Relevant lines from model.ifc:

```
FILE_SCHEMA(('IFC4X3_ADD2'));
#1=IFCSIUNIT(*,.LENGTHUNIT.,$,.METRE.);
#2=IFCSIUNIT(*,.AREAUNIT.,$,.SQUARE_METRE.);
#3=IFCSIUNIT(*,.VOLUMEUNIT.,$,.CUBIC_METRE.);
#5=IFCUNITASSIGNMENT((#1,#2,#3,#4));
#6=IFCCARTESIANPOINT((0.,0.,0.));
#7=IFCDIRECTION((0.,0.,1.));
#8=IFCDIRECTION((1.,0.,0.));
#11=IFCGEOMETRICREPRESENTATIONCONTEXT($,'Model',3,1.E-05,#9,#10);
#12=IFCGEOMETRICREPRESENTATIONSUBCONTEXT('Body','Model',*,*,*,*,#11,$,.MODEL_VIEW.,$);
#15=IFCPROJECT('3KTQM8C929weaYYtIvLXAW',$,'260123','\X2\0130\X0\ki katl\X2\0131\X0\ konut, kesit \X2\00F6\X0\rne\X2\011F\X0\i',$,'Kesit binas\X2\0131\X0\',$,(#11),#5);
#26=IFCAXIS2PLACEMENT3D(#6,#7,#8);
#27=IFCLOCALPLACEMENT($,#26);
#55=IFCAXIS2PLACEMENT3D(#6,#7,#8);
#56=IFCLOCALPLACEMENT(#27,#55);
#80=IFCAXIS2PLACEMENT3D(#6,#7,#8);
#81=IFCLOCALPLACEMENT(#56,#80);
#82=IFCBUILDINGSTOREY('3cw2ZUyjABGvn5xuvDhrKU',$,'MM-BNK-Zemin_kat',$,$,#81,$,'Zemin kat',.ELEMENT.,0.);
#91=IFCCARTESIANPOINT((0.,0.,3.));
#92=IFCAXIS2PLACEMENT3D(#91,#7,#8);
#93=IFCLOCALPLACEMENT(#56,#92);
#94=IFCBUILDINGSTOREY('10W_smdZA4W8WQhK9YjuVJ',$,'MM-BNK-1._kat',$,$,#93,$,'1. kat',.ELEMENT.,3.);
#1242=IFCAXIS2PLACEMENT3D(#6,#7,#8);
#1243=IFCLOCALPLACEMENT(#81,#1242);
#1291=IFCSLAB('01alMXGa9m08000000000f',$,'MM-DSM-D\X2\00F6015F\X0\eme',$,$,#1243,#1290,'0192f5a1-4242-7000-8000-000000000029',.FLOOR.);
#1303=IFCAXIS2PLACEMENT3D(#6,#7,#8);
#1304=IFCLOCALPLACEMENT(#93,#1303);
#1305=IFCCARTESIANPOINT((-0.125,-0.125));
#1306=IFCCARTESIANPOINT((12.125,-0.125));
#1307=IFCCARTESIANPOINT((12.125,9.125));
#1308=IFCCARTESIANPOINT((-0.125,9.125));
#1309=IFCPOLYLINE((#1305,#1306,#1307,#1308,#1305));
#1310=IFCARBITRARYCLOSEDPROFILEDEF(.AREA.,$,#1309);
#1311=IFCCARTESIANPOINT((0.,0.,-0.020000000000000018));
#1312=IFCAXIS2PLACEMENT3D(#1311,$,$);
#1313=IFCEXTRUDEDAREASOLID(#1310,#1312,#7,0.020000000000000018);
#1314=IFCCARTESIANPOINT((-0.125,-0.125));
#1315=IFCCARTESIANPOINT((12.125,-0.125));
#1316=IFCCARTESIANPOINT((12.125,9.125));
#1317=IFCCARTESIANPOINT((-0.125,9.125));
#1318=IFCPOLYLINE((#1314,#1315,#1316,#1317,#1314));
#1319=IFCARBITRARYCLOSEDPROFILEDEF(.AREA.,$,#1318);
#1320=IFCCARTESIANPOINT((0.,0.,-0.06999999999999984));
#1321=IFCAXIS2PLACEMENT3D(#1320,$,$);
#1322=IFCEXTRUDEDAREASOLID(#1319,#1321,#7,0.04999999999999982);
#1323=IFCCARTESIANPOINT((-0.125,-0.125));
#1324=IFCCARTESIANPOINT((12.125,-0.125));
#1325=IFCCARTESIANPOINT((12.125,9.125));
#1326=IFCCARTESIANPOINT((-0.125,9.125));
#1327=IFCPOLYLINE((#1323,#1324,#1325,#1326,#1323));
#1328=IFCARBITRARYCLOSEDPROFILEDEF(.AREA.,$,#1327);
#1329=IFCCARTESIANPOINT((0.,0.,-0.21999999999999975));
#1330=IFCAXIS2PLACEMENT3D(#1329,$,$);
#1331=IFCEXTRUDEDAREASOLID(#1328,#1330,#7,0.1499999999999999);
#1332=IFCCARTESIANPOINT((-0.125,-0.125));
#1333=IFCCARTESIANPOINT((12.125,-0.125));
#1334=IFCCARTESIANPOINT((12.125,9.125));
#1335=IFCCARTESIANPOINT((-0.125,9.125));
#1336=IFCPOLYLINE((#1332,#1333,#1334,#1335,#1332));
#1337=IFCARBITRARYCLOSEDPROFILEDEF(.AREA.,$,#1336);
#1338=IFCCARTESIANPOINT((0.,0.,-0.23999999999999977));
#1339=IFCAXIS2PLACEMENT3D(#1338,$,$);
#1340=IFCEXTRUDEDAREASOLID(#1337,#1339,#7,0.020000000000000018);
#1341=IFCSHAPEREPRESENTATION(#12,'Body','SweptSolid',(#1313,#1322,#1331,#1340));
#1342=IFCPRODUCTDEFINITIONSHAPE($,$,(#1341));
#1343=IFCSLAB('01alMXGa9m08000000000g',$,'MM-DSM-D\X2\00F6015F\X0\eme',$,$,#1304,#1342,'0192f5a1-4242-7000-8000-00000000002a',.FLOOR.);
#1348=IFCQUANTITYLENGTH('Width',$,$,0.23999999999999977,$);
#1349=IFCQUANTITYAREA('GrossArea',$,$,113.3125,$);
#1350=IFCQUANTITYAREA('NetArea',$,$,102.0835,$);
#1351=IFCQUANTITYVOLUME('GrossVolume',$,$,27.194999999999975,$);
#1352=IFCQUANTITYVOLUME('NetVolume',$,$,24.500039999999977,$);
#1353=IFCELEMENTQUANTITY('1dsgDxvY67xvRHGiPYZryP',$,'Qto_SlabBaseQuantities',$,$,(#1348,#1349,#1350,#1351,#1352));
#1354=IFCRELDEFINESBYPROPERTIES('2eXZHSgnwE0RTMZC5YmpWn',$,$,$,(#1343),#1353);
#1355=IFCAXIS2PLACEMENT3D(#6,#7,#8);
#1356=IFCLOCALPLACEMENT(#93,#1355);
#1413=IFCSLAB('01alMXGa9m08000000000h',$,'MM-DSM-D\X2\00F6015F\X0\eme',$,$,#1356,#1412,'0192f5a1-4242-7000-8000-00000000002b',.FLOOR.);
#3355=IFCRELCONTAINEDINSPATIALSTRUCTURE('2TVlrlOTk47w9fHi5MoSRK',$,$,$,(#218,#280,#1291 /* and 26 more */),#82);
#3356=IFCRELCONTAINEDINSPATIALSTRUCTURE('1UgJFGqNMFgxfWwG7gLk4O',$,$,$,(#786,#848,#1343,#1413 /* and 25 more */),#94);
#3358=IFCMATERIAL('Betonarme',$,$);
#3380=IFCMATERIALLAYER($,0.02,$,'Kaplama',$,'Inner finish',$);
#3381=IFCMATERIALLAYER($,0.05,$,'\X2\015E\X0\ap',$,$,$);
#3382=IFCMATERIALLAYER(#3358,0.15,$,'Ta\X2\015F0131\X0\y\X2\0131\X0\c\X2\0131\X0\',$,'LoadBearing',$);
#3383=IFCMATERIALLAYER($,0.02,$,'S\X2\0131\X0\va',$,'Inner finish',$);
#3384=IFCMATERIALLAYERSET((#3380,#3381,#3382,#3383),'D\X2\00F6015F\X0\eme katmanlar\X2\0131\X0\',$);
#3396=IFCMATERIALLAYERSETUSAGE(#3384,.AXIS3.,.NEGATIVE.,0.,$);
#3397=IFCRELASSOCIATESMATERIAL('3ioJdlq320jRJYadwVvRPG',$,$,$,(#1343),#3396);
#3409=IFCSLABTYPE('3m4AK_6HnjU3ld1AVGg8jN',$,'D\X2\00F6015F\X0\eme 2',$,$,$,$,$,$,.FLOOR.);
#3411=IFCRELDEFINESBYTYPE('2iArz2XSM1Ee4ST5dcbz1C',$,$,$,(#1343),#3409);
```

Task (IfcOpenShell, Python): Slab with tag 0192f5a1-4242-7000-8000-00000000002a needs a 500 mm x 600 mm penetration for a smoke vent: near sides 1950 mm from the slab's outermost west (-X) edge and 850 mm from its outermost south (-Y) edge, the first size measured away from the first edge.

```python
import numpy as np
import ifcopenshell
import ifcopenshell.api.feature
import ifcopenshell.api.geometry
import ifcopenshell.api.pset
import ifcopenshell.api.root
import ifcopenshell.geom
import ifcopenshell.util.element
import ifcopenshell.util.placement
import ifcopenshell.util.representation
import ifcopenshell.util.shape
import ifcopenshell.util.unit

model = ifcopenshell.open("model.ifc")
unit_scale = ifcopenshell.util.unit.calculate_unit_scale(model)
area_scale = ifcopenshell.util.unit.calculate_unit_scale(model, "AREAUNIT")
volume_scale = ifcopenshell.util.unit.calculate_unit_scale(model, "VOLUMEUNIT")
settings = ifcopenshell.geom.settings()


def volume(element):
    """Net volume in cubic metres, openings subtracted."""
    shape = ifcopenshell.geom.create_shape(settings, element)
    return ifcopenshell.util.shape.get_volume(shape.geometry)


slab = model.by_guid("01alMXGa9m08000000000g")
before = volume(slab)

# Extent in the slab's own axes, in metres. The edges named are its -X and -Y sides.
slab_shape = ifcopenshell.geom.create_shape(settings, slab)
vertices = ifcopenshell.util.shape.get_vertices(slab_shape.geometry)
x_min, y_min, bottom = vertices.min(axis=0)
top = vertices[:, 2].max()

opening = ifcopenshell.api.root.create_entity(model, ifc_class="IfcOpeningElement", name="Smoke vent opening", predefined_type="OPENING")
context = ifcopenshell.util.representation.get_context(model, "Model", "Body", "MODEL_VIEW")
width, depth = 0.5, 0.6
outline = [(0.0, 0.0), (width, 0.0), (width, depth), (0.0, depth), (0.0, 0.0)]
# Overshoot both faces by 50 mm so the cut is clean.
shape = ifcopenshell.api.geometry.add_slab_representation(
    model, context=context, depth=top - bottom + 0.1, polyline=outline
)
ifcopenshell.api.geometry.assign_representation(model, product=opening, representation=shape)

matrix = ifcopenshell.util.placement.get_local_placement(slab.ObjectPlacement)
matrix[:, 3] = matrix @ np.append(np.array([x_min + 1.95, y_min + 0.85, bottom - 0.05]) / unit_scale, 1.0)
ifcopenshell.api.geometry.edit_object_placement(model, product=opening, matrix=matrix, is_si=False)
ifcopenshell.api.feature.add_feature(model, feature=opening, element=slab)

after = volume(slab)

# Update the slab's stored quantities.
qto = model.by_id(ifcopenshell.util.element.get_pset(slab, "Qto_SlabBaseQuantities", should_inherit=False)["id"])
ifcopenshell.api.pset.edit_qto(model, qto=qto, properties={
    "NetArea": after / (top - bottom) / area_scale,
    "NetVolume": after / volume_scale,
})

print(f"slab volume {before:.3f} -> {after:.3f} m3")

model.write("model_edited.ifc")
```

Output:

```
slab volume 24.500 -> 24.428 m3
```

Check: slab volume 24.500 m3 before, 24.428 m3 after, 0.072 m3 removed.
